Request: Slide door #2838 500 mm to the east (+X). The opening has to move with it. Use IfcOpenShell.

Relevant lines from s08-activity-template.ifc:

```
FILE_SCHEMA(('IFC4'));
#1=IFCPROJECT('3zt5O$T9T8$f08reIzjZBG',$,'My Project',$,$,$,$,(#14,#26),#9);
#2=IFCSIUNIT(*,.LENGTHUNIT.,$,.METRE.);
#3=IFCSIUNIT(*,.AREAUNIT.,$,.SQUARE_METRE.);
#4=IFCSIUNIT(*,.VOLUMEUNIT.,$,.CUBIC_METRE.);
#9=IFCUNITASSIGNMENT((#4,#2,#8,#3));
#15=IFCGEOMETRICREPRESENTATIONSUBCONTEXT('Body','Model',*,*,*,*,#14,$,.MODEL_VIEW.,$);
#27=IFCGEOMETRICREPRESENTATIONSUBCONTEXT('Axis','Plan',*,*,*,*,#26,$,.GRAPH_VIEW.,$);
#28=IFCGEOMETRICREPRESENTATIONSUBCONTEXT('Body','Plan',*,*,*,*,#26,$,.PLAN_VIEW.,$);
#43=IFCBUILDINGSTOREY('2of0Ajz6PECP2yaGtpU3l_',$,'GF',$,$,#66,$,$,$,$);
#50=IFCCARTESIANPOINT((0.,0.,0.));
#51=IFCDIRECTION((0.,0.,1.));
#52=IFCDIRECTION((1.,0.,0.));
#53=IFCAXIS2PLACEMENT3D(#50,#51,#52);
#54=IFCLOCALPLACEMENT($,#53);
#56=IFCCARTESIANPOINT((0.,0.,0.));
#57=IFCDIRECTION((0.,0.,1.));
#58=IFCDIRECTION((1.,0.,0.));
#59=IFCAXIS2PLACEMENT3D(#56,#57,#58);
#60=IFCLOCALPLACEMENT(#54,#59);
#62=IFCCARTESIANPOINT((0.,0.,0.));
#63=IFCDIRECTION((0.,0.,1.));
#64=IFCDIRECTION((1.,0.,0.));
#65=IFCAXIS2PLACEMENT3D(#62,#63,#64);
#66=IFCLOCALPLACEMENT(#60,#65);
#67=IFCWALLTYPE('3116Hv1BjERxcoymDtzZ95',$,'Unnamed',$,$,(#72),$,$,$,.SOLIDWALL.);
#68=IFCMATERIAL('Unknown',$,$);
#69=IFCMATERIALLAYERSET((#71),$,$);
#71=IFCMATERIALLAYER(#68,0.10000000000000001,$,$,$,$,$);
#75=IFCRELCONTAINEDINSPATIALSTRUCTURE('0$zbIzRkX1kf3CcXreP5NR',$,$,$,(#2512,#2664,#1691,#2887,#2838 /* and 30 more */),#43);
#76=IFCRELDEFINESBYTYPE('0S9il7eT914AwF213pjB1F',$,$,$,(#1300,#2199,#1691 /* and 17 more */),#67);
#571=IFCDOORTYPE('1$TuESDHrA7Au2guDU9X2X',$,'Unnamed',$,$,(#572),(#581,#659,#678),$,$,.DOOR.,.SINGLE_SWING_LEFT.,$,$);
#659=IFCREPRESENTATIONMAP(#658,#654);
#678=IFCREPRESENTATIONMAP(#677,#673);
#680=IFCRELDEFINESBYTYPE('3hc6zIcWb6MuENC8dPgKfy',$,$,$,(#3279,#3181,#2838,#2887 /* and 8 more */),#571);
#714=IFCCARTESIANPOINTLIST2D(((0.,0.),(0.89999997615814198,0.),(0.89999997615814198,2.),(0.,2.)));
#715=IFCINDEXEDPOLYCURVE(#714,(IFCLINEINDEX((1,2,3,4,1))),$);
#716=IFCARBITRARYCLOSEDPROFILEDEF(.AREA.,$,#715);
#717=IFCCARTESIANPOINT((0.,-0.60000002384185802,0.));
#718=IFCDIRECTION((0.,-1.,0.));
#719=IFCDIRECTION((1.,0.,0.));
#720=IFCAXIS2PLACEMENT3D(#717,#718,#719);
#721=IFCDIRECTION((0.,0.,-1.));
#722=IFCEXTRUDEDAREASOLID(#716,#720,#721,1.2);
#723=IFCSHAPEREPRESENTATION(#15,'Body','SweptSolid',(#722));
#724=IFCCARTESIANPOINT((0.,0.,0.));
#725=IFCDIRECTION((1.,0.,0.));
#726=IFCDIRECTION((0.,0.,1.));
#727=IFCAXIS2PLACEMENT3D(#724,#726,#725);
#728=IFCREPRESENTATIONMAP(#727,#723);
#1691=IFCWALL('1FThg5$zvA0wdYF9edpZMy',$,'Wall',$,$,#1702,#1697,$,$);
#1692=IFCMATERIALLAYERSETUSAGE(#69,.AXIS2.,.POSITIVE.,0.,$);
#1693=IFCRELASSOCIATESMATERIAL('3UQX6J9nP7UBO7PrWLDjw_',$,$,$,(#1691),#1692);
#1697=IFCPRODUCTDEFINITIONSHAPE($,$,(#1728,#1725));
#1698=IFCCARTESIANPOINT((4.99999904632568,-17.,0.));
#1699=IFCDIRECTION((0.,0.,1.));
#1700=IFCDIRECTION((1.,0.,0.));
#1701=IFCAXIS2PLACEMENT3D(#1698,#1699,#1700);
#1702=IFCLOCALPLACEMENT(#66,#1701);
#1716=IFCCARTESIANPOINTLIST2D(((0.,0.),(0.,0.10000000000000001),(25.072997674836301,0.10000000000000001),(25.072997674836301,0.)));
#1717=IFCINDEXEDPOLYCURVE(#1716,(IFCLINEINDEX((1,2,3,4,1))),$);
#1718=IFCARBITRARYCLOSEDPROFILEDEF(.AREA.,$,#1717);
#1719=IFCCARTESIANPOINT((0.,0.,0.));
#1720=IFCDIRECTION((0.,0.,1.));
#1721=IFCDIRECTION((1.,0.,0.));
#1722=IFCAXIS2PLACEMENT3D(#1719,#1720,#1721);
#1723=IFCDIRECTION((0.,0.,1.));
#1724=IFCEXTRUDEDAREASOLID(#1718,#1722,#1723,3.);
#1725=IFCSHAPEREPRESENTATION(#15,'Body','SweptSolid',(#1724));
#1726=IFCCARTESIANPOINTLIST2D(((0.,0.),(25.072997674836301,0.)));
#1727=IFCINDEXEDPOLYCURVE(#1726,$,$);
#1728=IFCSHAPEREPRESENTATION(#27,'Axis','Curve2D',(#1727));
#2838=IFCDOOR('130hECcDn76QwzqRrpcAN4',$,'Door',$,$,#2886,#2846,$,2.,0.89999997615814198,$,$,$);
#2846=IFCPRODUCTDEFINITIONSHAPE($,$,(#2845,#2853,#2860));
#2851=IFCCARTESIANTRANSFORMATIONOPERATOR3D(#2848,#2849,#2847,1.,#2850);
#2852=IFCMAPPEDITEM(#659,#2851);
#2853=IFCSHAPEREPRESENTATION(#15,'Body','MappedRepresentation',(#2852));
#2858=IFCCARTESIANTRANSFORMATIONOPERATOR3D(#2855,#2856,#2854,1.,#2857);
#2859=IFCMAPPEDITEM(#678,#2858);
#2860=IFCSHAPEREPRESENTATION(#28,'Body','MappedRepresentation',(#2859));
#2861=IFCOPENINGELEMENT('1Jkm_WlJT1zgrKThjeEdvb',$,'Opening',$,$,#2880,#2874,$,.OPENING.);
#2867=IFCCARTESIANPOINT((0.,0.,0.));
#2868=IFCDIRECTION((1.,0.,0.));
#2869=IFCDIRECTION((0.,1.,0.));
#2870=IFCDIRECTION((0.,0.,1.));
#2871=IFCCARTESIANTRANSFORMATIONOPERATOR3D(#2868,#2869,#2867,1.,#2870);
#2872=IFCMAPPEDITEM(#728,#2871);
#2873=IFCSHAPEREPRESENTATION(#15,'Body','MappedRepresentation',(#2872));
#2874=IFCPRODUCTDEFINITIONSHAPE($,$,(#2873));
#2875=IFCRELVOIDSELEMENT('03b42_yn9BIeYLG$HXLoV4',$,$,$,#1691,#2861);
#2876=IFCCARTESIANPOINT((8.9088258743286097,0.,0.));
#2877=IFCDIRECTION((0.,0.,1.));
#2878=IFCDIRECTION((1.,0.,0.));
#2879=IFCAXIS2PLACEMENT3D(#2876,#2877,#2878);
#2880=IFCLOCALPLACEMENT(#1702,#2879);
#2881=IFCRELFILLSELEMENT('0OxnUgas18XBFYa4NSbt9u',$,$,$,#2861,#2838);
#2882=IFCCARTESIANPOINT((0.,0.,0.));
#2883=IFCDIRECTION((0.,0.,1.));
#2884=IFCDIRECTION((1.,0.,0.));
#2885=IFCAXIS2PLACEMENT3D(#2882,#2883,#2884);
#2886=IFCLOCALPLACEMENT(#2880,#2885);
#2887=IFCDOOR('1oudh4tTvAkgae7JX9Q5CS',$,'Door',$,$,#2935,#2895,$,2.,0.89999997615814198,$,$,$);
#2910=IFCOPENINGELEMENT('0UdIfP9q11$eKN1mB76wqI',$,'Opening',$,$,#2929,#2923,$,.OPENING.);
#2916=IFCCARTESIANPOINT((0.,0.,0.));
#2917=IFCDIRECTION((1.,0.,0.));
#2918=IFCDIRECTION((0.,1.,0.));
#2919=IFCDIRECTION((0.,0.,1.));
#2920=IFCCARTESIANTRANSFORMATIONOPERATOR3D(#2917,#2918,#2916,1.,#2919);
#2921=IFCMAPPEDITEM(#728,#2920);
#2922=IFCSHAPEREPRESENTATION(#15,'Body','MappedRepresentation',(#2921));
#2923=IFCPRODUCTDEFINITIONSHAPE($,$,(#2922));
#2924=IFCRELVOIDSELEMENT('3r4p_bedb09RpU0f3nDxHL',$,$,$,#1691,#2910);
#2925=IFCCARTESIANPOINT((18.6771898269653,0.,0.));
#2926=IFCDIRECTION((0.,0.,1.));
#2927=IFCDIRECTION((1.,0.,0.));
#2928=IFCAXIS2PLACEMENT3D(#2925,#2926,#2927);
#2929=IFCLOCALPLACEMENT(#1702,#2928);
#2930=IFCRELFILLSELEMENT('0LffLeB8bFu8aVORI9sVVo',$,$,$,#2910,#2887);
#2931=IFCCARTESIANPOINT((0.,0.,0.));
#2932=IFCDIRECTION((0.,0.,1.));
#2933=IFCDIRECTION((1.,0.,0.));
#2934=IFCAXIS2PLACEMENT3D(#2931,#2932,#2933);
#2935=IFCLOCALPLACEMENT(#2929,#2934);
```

```python
import ifcopenshell
import ifcopenshell.api.geometry
import ifcopenshell.util.placement

model = ifcopenshell.open("s08-activity-template.ifc")

door = model.by_guid("130hECcDn76QwzqRrpcAN4")
opening = door.FillsVoids[0].RelatingOpeningElement
wall = opening.VoidsElements[0].RelatingBuildingElement

wall_matrix = ifcopenshell.util.placement.get_local_placement(wall.ObjectPlacement)
shift = wall_matrix[:3, 0] * 0.5
before = ifcopenshell.util.placement.get_local_placement(door.ObjectPlacement)[:3, 3].copy()

# The door is placed relative to its opening, so it follows when the opening moves.
matrix = ifcopenshell.util.placement.get_local_placement(opening.ObjectPlacement)
matrix[:3, 3] += shift
ifcopenshell.api.geometry.edit_object_placement(
    model, product=opening, matrix=matrix, is_si=False, should_transform_children=True
)

after = ifcopenshell.util.placement.get_local_placement(door.ObjectPlacement)[:3, 3]
print("door moved by", (after - before).round(3) + 0.0)

model.write("s08-activity-template_updated.ifc")
```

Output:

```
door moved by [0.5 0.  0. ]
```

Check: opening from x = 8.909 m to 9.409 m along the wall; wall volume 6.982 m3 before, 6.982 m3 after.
